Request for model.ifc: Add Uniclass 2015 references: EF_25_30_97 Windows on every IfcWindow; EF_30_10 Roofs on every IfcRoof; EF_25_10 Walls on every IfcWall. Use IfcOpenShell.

First a look at what the model holds.

```python
import ifcopenshell

model = ifcopenshell.open("model.ifc")
print(model.schema)
print("classifications:", [c.Name for c in model.by_type("IfcClassification")])
for ifc_class in ("IfcDoor", "IfcRoof", "IfcStair", "IfcWall", "IfcWindow"):
    print(ifc_class, len(model.by_type(ifc_class)))
```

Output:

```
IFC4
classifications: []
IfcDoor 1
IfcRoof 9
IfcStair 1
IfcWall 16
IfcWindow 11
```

```python
import ifcopenshell
import ifcopenshell.api.classification

model = ifcopenshell.open("model.ifc")

system = ifcopenshell.api.classification.add_classification(model, classification="Uniclass 2015")

codes = {
    "IfcWindow": ("EF_25_30_97", "Windows"),
    "IfcRoof": ("EF_30_10", "Roofs"),
    "IfcWall": ("EF_25_10", "Walls"),
}
for ifc_class, (code, name) in codes.items():
    products = model.by_type(ifc_class)
    ifcopenshell.api.classification.add_reference(
        model, products=products, classification=system, identification=code, name=name
    )
    print(code, len(products))

model.write("model_updated.ifc")
```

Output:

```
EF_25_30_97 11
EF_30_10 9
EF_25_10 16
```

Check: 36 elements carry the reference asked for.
